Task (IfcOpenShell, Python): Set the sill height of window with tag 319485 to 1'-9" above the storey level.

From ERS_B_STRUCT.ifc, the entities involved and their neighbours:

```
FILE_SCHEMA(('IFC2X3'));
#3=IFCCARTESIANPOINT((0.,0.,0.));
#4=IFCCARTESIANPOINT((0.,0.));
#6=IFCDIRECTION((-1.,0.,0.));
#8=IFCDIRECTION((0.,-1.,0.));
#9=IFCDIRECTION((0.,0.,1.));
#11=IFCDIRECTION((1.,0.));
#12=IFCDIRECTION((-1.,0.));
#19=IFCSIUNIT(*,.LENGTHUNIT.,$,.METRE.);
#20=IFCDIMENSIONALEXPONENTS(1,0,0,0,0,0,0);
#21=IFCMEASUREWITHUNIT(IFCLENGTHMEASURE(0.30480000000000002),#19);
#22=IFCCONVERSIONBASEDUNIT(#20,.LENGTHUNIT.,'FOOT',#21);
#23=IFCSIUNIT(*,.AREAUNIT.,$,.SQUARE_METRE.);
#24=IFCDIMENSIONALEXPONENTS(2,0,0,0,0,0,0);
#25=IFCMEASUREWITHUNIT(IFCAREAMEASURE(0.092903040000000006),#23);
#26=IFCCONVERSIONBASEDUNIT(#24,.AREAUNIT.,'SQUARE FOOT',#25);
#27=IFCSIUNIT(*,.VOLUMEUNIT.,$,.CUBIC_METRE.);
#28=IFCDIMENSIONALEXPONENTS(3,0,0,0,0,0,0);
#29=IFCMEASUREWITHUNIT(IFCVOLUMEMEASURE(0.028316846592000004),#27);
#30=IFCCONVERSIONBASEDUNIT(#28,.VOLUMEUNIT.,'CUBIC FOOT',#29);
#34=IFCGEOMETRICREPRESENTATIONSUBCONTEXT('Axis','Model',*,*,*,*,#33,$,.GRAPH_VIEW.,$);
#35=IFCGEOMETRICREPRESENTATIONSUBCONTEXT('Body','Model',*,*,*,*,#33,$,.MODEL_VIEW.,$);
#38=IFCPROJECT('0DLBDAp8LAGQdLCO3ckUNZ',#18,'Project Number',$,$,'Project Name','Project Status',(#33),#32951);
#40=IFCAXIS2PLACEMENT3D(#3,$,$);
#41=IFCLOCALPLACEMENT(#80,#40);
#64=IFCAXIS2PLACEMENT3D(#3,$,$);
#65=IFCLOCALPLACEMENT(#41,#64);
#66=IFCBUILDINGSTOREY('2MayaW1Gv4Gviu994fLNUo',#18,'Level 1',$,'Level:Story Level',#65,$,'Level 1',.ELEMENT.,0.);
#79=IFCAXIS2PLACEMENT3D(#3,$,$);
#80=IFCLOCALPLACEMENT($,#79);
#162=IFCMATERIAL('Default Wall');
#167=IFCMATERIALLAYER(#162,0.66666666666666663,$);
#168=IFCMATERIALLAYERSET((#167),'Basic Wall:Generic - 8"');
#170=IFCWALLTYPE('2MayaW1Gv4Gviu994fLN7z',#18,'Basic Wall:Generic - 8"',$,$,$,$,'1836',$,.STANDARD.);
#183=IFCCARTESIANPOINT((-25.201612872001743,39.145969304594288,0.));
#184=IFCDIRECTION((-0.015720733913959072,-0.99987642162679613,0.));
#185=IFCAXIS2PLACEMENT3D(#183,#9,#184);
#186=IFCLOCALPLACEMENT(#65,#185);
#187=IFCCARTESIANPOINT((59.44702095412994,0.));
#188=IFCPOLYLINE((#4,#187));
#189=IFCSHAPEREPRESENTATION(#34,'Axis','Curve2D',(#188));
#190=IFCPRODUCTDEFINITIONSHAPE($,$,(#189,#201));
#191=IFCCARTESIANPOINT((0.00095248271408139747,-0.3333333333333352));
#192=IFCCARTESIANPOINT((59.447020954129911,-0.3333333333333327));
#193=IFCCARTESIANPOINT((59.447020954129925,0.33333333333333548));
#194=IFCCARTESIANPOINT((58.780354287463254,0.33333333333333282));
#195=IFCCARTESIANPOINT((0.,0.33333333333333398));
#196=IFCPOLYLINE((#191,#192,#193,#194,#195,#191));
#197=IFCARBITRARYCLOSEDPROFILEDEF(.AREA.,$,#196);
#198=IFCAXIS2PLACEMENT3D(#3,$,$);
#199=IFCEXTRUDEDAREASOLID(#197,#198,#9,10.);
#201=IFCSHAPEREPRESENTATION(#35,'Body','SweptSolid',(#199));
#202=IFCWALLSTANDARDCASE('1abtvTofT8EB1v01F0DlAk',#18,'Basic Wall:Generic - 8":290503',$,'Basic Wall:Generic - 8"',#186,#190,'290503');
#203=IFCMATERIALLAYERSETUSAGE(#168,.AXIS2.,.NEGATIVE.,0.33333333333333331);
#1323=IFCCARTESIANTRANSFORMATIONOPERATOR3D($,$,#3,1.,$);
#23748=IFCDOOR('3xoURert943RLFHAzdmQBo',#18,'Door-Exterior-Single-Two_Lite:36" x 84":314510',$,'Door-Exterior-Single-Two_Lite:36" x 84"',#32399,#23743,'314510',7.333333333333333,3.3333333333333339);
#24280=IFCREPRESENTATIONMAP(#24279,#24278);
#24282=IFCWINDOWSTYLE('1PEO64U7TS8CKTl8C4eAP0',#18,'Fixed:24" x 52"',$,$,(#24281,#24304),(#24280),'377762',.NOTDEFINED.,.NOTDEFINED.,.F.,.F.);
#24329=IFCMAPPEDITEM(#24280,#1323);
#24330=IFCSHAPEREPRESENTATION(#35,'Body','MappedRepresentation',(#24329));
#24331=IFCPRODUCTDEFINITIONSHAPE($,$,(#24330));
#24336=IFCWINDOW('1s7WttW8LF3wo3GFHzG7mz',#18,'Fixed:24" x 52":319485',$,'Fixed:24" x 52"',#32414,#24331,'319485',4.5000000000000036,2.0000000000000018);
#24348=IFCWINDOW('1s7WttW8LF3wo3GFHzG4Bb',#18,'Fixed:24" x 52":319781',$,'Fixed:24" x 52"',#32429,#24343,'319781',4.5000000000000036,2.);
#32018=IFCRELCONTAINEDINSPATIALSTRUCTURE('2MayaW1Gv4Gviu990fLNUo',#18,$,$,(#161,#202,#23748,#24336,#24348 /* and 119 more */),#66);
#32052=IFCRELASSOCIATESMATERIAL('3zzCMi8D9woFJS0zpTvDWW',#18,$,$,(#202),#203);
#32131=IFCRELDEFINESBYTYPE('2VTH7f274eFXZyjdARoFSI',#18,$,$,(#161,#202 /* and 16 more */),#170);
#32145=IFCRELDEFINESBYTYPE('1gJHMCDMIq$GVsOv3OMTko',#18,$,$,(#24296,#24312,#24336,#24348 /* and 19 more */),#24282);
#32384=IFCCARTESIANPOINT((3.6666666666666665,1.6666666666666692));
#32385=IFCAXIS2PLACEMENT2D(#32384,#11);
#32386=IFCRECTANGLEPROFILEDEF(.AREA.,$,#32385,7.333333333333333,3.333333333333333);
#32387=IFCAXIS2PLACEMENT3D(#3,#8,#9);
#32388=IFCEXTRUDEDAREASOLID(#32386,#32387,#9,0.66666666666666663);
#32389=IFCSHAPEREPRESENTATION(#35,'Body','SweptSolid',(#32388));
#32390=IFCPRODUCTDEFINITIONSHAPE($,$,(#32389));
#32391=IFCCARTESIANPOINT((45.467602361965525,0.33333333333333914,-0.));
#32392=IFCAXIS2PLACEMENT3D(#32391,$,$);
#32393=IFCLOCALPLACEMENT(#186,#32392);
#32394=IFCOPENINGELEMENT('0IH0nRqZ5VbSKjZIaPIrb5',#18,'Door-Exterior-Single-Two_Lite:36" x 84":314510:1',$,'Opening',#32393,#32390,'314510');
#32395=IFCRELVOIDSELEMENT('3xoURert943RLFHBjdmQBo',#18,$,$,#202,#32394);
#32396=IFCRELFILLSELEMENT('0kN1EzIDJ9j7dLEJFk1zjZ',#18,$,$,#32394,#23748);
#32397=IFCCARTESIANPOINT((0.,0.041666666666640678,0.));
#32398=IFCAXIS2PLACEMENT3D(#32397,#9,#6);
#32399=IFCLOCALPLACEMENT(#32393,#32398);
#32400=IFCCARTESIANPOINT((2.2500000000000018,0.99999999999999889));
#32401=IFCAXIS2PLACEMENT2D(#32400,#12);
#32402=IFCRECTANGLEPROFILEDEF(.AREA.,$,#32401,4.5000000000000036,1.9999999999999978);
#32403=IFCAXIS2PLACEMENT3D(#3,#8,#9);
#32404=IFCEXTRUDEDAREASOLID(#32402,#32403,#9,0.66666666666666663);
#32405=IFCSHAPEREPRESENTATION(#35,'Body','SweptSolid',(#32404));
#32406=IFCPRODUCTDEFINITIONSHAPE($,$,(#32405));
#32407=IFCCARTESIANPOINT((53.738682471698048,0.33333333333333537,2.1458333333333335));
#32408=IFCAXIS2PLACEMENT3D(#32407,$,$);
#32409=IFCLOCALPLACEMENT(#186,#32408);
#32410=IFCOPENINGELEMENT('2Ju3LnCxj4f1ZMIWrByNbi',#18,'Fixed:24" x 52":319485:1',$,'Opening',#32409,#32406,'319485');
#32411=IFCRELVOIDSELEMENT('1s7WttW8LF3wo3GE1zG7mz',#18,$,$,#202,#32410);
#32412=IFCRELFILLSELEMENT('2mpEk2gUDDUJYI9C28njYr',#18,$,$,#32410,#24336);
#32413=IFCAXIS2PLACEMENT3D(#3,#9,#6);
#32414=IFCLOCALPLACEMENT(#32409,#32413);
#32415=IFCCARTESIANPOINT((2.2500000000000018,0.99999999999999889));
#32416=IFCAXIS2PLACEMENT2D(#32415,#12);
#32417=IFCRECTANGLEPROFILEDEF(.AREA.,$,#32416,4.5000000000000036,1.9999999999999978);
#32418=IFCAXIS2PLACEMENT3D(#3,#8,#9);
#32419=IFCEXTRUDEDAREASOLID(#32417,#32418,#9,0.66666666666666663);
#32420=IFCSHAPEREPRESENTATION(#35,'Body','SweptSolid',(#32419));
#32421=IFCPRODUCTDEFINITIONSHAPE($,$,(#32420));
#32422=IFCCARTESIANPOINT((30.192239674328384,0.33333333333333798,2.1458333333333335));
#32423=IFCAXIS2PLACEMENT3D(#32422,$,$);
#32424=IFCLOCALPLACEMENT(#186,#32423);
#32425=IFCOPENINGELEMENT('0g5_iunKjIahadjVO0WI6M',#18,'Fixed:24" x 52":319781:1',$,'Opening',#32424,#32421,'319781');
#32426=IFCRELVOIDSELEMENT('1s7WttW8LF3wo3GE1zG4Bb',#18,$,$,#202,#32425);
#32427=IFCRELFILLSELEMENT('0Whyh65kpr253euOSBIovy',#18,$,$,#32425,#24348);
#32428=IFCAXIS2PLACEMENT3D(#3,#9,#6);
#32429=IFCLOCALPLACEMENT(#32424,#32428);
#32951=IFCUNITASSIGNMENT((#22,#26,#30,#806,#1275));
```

```python
import numpy as np
import ifcopenshell
import ifcopenshell.api.geometry
import ifcopenshell.geom
import ifcopenshell.util.element
import ifcopenshell.util.placement
import ifcopenshell.util.shape
import ifcopenshell.util.unit

model = ifcopenshell.open("ERS_B_STRUCT.ifc")
unit_scale = ifcopenshell.util.unit.calculate_unit_scale(model)

window = model.by_guid("1s7WttW8LF3wo3GFHzG7mz")
opening = window.FillsVoids[0].RelatingOpeningElement
storey = ifcopenshell.util.element.get_container(window, ifc_class="IfcBuildingStorey")
level = ifcopenshell.util.placement.get_local_placement(storey.ObjectPlacement)[2, 3]

# The opening's origin need not be at the sill, so measure its lowest point.
shape = ifcopenshell.geom.create_shape(ifcopenshell.geom.settings(), opening)
bottom = ifcopenshell.util.shape.get_shape_bottom_elevation(shape, shape.geometry) / unit_scale
dz = level + 21 * 0.0254 / unit_scale - bottom

shift = np.array([0.0, 0.0, dz])
# The window is placed relative to its opening, so it follows when the opening moves.
matrix = ifcopenshell.util.placement.get_local_placement(opening.ObjectPlacement)
matrix[:3, 3] += shift
ifcopenshell.api.geometry.edit_object_placement(
    model, product=opening, matrix=matrix, is_si=False, should_transform_children=True
)

print(f"moved by {dz * unit_scale:+.3f} m")

model.write("ERS_B_STRUCT_rev.ifc")
```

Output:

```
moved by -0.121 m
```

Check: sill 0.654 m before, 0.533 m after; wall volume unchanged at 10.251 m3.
